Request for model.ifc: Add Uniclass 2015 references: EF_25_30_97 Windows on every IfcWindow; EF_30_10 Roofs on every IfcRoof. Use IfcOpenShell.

First a look at what the model holds.

```python
import ifcopenshell

model = ifcopenshell.open("model.ifc")
print(model.schema)
print("classifications:", [c.Name for c in model.by_type("IfcClassification")])
for ifc_class in ("IfcDoor", "IfcRoof", "IfcStair", "IfcWall", "IfcWindow"):
    print(ifc_class, len(model.by_type(ifc_class)))
```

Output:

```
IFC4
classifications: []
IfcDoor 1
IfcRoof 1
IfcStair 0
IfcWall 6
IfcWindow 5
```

```python
import ifcopenshell
import ifcopenshell.api.classification

model = ifcopenshell.open("model.ifc")

system = ifcopenshell.api.classification.add_classification(model, classification="Uniclass 2015")

codes = {
    "IfcWindow": ("EF_25_30_97", "Windows"),
    "IfcRoof": ("EF_30_10", "Roofs"),
}
for ifc_class, (code, name) in codes.items():
    products = model.by_type(ifc_class)
    ifcopenshell.api.classification.add_reference(
        model, products=products, classification=system, identification=code, name=name
    )
    print(code, len(products))

model.write("model-out.ifc")
```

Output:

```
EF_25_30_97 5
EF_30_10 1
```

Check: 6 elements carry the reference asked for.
